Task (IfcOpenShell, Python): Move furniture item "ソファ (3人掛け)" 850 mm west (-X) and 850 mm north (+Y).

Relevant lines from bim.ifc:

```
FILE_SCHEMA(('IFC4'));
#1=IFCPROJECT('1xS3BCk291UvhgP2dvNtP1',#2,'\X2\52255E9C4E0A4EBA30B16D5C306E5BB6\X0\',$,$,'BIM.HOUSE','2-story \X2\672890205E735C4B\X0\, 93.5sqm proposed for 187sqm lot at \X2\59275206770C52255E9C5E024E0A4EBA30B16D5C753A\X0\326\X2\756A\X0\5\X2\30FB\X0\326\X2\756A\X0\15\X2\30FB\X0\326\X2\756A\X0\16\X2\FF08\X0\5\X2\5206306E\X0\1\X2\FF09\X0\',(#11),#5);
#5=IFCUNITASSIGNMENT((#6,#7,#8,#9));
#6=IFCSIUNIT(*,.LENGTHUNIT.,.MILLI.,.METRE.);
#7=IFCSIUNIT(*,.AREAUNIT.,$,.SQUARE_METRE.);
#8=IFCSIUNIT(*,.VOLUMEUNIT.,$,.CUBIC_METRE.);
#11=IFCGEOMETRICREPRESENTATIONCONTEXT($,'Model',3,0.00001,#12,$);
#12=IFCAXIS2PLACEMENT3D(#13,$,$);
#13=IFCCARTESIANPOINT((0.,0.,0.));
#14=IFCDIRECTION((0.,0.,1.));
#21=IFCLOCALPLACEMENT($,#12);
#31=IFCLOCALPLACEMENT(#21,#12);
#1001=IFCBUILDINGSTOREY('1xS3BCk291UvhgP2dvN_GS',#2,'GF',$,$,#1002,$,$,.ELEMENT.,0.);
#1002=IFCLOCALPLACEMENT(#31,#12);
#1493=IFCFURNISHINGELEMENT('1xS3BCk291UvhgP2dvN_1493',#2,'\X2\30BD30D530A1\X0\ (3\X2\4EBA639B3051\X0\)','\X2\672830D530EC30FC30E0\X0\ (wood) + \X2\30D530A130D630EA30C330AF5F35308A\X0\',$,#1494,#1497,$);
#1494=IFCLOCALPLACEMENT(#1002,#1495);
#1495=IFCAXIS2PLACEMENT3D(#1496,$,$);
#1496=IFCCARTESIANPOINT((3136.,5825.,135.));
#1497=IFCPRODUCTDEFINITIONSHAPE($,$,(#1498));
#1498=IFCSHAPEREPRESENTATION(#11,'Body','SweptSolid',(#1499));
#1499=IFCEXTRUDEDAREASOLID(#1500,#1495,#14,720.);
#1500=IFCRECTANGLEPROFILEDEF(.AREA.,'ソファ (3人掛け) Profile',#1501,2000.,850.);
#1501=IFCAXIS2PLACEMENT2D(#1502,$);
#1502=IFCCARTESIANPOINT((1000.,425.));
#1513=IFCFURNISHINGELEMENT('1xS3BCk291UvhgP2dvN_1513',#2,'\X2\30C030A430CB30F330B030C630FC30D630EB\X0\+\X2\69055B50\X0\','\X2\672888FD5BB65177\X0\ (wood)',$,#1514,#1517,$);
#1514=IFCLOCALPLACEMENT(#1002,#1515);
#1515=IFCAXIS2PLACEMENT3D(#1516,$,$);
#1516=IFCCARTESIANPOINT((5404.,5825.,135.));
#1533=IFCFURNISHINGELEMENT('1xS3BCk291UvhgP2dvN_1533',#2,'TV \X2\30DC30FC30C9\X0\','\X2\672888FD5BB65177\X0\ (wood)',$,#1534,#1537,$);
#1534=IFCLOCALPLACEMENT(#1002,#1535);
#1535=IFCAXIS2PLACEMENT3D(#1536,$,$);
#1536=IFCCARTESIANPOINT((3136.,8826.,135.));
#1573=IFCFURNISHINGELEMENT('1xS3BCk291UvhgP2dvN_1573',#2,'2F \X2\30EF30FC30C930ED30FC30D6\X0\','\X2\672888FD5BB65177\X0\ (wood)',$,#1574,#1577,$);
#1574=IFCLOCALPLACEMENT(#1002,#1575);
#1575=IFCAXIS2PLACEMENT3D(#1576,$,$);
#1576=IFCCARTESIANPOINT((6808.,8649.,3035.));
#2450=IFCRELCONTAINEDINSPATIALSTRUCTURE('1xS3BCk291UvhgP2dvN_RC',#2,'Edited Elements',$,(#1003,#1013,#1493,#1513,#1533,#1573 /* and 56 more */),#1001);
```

```python
import ifcopenshell
import ifcopenshell.api.geometry
import ifcopenshell.util.placement
import ifcopenshell.util.unit

model = ifcopenshell.open("bim.ifc")
unit_scale = ifcopenshell.util.unit.calculate_unit_scale(model)

item = model.by_guid("1xS3BCk291UvhgP2dvN_1493")
matrix = ifcopenshell.util.placement.get_local_placement(item.ObjectPlacement)
matrix[0, 3] -= 0.85 / unit_scale
matrix[1, 3] += 0.85 / unit_scale
ifcopenshell.api.geometry.edit_object_placement(model, product=item, matrix=matrix, is_si=False)

print(ifcopenshell.util.placement.get_local_placement(item.ObjectPlacement).round(3) + 0.0)

model.write("bim_edited.ifc")
```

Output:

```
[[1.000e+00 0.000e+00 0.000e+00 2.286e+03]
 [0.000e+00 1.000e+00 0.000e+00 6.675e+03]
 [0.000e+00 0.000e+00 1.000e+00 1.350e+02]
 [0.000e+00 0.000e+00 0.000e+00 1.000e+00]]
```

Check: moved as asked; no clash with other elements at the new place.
